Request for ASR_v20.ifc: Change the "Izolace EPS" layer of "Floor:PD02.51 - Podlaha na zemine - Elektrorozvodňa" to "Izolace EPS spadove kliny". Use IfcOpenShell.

First a look at what the model holds.

```python
import ifcopenshell
import ifcopenshell.util.element

model = ifcopenshell.open("ASR_v20.ifc")
print(model.schema)
for layer_set in model.by_type("IfcMaterialLayerSet"):
    if layer_set.LayerSetName == "Floor:PD02.51 - Podlaha na zemine - Elektrorozvodňa":
        for layer in layer_set.MaterialLayers:
            print(layer.id(), layer.Material and layer.Material.Name, layer.LayerThickness, sep=" | ")
        print(len(ifcopenshell.util.element.get_elements_by_material(model, layer_set)), "elements and types use it")
print(sorted(m.Name for m in model.by_type("IfcMaterial") if m.Name)[:60])
```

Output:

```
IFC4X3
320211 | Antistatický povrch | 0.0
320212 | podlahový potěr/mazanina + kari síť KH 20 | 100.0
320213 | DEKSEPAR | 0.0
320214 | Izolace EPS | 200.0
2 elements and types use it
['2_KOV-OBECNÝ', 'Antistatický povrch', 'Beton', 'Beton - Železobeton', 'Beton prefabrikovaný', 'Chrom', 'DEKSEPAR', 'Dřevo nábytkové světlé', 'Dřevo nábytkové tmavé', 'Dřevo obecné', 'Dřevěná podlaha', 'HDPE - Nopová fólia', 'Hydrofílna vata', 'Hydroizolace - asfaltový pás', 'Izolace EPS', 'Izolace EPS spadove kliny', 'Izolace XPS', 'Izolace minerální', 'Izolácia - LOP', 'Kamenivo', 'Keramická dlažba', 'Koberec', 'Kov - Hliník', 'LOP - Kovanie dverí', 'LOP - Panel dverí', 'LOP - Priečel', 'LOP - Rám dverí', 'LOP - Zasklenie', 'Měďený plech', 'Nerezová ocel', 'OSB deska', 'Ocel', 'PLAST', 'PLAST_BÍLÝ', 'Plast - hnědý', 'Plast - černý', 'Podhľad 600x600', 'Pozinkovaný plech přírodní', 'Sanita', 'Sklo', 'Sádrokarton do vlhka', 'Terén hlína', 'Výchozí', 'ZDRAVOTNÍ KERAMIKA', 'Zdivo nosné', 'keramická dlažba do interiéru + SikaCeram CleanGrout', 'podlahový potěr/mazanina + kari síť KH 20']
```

```python
import ifcopenshell
import ifcopenshell.api.material

model = ifcopenshell.open("ASR_v20.ifc")

layer_set = next(s for s in model.by_type("IfcMaterialLayerSet") if s.LayerSetName == "Floor:PD02.51 - Podlaha na zemine - Elektrorozvodňa")
layer = next(l for l in layer_set.MaterialLayers if l.Material and l.Material.Name == "Izolace EPS")
material = next(m for m in model.by_type("IfcMaterial") if m.Name == "Izolace EPS spadove kliny")

# Point this one layer at the other material; renaming the old one would change it everywhere.
ifcopenshell.api.material.edit_layer(model, layer=layer, attributes={"Name": material.Name}, material=material)

print([l.Material.Name if l.Material else None for l in layer_set.MaterialLayers])

model.write("ASR_v20_v2.ifc")
```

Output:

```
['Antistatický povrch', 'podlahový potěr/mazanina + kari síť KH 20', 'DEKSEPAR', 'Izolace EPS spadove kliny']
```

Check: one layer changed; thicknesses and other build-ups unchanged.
